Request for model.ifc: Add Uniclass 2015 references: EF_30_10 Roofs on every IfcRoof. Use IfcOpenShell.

First a look at what the model holds.

```python
import ifcopenshell

model = ifcopenshell.open("model.ifc")
print(model.schema)
print("classifications:", [c.Name for c in model.by_type("IfcClassification")])
for ifc_class in ("IfcDoor", "IfcRoof", "IfcStair", "IfcWall", "IfcWindow"):
    print(ifc_class, len(model.by_type(ifc_class)))
```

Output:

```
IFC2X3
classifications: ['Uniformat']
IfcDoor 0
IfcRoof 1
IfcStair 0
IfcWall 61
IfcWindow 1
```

```python
import ifcopenshell
import ifcopenshell.api.classification

model = ifcopenshell.open("model.ifc")

# IFC2X3 requires Source and Edition and has no link from the project to the system.
system = model.create_entity("IfcClassification", Source="NBS", Edition="2015", Name="Uniclass 2015")

codes = {
    "IfcRoof": ("EF_30_10", "Roofs"),
}
for ifc_class, (code, name) in codes.items():
    products = model.by_type(ifc_class)
    ifcopenshell.api.classification.add_reference(
        model, products=products, classification=system, identification=code, name=name
    )
    print(code, len(products))

model.write("model_updated.ifc")
```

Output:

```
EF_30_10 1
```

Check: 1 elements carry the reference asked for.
